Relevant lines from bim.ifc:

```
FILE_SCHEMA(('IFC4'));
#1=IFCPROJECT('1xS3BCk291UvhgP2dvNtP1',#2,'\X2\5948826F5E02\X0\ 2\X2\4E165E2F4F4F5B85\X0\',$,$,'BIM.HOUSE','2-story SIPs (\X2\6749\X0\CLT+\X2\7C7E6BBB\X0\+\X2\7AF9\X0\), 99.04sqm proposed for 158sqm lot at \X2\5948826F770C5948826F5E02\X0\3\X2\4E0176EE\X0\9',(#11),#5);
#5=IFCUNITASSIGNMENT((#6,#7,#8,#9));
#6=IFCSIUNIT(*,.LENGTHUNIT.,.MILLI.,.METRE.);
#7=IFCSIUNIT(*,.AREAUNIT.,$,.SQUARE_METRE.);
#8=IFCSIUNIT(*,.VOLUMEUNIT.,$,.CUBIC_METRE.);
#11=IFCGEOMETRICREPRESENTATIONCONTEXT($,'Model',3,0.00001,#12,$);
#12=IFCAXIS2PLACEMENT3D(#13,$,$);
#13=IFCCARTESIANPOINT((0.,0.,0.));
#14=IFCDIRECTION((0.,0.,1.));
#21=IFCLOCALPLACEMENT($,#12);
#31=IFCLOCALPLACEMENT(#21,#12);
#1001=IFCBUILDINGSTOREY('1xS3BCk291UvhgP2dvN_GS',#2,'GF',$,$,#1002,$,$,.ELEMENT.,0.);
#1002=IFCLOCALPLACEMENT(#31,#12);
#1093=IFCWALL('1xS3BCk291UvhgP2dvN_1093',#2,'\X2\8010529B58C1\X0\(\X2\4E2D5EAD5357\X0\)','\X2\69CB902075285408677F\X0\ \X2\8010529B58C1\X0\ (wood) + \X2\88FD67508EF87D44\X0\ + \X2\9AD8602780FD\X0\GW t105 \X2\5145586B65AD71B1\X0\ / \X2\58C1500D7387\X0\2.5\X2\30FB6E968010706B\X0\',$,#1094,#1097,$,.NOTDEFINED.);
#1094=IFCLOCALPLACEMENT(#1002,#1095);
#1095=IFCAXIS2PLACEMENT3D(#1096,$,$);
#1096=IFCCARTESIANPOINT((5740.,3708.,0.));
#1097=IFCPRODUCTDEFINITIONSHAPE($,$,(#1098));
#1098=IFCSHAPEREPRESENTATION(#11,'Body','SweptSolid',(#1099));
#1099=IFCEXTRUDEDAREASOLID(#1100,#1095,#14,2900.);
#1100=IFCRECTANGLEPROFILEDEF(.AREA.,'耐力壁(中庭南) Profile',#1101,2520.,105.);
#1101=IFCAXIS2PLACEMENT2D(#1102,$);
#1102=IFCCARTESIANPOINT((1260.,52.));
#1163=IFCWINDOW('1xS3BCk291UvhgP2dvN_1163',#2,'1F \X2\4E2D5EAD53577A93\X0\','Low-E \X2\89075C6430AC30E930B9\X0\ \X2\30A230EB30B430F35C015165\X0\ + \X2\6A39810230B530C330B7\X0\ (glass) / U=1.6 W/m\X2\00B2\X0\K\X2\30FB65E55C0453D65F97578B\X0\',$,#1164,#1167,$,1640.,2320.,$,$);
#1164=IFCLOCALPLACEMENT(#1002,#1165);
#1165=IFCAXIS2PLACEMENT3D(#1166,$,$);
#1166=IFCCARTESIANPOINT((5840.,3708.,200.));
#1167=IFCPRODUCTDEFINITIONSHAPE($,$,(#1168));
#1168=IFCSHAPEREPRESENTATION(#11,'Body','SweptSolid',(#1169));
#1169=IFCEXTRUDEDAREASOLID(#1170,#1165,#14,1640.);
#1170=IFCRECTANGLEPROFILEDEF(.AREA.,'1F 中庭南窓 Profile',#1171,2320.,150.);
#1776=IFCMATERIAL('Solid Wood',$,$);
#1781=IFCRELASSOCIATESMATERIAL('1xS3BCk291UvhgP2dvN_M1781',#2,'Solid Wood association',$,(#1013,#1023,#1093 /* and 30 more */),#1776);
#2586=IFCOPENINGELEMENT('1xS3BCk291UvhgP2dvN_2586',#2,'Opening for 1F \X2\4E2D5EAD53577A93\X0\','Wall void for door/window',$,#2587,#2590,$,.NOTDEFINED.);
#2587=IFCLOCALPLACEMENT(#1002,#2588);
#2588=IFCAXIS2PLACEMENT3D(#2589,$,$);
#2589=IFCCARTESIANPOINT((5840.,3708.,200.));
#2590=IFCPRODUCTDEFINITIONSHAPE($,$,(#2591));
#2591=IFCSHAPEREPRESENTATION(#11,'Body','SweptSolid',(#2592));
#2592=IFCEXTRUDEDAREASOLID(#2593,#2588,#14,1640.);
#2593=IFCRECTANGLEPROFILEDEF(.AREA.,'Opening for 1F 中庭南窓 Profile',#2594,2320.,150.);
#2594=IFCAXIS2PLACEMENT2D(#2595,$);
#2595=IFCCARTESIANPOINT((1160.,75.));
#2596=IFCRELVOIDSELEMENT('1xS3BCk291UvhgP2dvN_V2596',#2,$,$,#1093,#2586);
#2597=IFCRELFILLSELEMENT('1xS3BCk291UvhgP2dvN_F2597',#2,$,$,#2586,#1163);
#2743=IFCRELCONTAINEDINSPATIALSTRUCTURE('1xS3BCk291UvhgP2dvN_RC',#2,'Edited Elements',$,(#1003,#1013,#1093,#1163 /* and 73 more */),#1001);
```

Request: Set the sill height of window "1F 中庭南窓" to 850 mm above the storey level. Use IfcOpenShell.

```python
import numpy as np
import ifcopenshell
import ifcopenshell.api.geometry
import ifcopenshell.geom
import ifcopenshell.util.element
import ifcopenshell.util.placement
import ifcopenshell.util.shape
import ifcopenshell.util.unit

model = ifcopenshell.open("bim.ifc")
unit_scale = ifcopenshell.util.unit.calculate_unit_scale(model)

window = model.by_guid("1xS3BCk291UvhgP2dvN_1163")
opening = window.FillsVoids[0].RelatingOpeningElement
storey = ifcopenshell.util.element.get_container(window, ifc_class="IfcBuildingStorey")
level = ifcopenshell.util.placement.get_local_placement(storey.ObjectPlacement)[2, 3]

# The opening's origin need not be at the sill, so measure its lowest point.
shape = ifcopenshell.geom.create_shape(ifcopenshell.geom.settings(), opening)
bottom = ifcopenshell.util.shape.get_shape_bottom_elevation(shape, shape.geometry) / unit_scale
dz = level + 0.85 / unit_scale - bottom

shift = np.array([0.0, 0.0, dz])
# The window is not placed relative to its opening, so move both.
for product in (opening, window):
    matrix = ifcopenshell.util.placement.get_local_placement(product.ObjectPlacement)
    matrix[:3, 3] += shift
    ifcopenshell.api.geometry.edit_object_placement(model, product=product, matrix=matrix, is_si=False)

print(f"moved by {dz * unit_scale:+.3f} m")

model.write("bim_updated.ifc")
```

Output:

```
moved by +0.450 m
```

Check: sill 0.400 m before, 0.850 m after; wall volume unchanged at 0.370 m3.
